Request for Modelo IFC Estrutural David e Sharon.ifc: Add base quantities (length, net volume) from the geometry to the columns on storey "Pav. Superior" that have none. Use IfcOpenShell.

First a look at what the model holds.

```python
import ifcopenshell
import ifcopenshell.util.element
import ifcopenshell.util.unit

model = ifcopenshell.open("Modelo IFC Estrutural David e Sharon.ifc")
print(model.schema)
for unit_type in ("LENGTHUNIT", "AREAUNIT", "VOLUMEUNIT"):
    print(unit_type, ifcopenshell.util.unit.calculate_unit_scale(model, unit_type))
storey = next(s for s in model.by_type("IfcBuildingStorey") if s.Name == "Pav. Superior")
columns = [e for e in ifcopenshell.util.element.get_decomposition(storey) if e.is_a("IfcColumn")]
for e in sorted(columns, key=lambda e: e.id()):
    print(e.id(), e.is_a(), e.Name, list(ifcopenshell.util.element.get_psets(e, qtos_only=True)), sep=" | ")
```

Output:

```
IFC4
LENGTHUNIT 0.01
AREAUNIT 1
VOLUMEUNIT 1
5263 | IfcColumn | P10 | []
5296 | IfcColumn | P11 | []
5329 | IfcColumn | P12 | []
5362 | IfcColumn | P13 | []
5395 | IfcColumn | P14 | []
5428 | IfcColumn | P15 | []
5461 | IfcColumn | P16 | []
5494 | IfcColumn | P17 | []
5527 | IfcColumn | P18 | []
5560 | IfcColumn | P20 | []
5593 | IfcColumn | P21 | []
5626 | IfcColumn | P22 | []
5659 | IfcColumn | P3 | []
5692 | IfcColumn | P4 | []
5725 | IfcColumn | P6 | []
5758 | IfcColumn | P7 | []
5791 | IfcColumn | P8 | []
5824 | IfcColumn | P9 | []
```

```python
import ifcopenshell
import ifcopenshell.api.pset
import ifcopenshell.geom
import ifcopenshell.util.element
import ifcopenshell.util.shape
import ifcopenshell.util.unit

model = ifcopenshell.open("Modelo IFC Estrutural David e Sharon.ifc")
unit_scale = ifcopenshell.util.unit.calculate_unit_scale(model)
volume_scale = ifcopenshell.util.unit.calculate_unit_scale(model, "VOLUMEUNIT")
settings = ifcopenshell.geom.settings()

storey = next(s for s in model.by_type("IfcBuildingStorey") if s.Name == "Pav. Superior")
columns = [e for e in ifcopenshell.util.element.get_decomposition(storey) if e.is_a("IfcColumn")]

for e in sorted(columns, key=lambda e: e.id()):
    if ifcopenshell.util.element.get_psets(e, qtos_only=True, should_inherit=False):
        continue
    # Geometry comes back in metres, in the element's own axes.
    shape = ifcopenshell.geom.create_shape(settings, e)
    values = {
        "Length": ifcopenshell.util.shape.get_z(shape.geometry) / unit_scale,
        "NetVolume": ifcopenshell.util.shape.get_volume(shape.geometry) / volume_scale,
    }
    qto = ifcopenshell.api.pset.add_qto(model, product=e, name="Qto_ColumnBaseQuantities")
    ifcopenshell.api.pset.edit_qto(model, qto=qto, properties=values)
    print(e.id(), {k: round(v, 3) for k, v in values.items()})

model.write("Modelo IFC Estrutural David e Sharon_rev.ifc")
```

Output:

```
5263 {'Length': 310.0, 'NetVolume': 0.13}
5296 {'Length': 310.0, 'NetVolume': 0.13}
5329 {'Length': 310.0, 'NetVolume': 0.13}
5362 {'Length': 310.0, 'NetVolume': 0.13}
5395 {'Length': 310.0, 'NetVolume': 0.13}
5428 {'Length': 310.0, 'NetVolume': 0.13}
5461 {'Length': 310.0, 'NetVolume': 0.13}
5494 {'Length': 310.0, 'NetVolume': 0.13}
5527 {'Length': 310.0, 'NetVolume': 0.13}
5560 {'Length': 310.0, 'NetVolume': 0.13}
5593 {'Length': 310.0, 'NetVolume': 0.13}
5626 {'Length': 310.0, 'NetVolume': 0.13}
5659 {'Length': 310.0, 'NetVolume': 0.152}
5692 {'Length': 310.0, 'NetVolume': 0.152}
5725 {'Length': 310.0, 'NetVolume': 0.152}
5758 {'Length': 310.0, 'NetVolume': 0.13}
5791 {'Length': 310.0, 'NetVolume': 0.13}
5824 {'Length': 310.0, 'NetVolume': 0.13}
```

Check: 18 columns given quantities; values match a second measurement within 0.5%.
